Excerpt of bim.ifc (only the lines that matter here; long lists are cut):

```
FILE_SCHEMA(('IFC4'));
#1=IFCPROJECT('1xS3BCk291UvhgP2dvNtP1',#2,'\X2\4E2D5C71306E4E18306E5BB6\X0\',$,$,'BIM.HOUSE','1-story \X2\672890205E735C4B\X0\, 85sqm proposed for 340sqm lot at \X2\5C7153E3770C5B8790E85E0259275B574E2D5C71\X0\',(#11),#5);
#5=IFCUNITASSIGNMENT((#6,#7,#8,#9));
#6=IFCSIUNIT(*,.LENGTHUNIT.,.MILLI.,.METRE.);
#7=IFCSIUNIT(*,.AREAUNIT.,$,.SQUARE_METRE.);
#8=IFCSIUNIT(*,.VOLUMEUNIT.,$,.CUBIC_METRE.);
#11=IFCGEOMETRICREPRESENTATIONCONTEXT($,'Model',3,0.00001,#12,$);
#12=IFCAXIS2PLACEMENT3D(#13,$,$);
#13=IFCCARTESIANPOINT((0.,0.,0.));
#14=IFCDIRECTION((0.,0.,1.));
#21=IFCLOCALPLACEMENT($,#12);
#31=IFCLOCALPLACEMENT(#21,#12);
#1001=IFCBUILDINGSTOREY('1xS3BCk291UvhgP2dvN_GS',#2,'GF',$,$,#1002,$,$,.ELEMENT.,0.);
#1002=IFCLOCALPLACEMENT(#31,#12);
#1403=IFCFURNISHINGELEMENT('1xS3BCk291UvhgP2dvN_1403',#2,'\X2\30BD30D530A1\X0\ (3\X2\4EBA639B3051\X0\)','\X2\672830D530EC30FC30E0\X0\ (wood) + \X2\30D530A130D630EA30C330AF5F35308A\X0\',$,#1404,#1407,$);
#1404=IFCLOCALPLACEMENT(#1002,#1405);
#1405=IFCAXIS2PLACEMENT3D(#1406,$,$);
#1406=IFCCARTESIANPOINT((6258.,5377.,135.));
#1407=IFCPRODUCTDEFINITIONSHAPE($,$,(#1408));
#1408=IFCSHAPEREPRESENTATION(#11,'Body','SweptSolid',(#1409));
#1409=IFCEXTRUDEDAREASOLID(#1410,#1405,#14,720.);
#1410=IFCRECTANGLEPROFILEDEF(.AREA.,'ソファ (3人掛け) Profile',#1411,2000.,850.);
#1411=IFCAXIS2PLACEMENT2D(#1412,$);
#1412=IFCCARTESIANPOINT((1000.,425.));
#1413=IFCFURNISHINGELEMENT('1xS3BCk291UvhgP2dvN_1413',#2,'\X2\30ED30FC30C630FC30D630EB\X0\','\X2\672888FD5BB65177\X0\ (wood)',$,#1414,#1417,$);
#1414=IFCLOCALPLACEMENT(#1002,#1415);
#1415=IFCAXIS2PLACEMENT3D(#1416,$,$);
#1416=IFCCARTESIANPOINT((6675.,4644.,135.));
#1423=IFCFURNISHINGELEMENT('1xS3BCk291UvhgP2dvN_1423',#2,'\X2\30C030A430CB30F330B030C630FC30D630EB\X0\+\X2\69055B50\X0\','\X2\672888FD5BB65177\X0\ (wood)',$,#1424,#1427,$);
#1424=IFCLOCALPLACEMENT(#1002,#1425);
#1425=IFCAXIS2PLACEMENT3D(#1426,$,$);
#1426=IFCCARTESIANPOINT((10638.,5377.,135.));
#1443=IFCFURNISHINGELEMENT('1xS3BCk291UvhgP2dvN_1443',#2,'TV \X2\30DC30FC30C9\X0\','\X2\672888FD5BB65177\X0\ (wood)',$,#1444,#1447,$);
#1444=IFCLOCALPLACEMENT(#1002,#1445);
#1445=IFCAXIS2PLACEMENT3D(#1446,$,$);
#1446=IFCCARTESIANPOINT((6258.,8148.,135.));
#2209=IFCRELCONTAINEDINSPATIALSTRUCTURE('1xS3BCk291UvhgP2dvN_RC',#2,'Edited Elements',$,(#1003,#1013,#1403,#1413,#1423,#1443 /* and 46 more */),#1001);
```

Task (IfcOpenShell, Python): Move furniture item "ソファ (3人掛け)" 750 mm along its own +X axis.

```python
import ifcopenshell
import ifcopenshell.api.geometry
import ifcopenshell.util.placement

model = ifcopenshell.open("bim.ifc")

item = model.by_guid("1xS3BCk291UvhgP2dvN_1403")
matrix = ifcopenshell.util.placement.get_local_placement(item.ObjectPlacement)
matrix[:3, 3] += matrix[:3, 0] * 750.0
ifcopenshell.api.geometry.edit_object_placement(model, product=item, matrix=matrix, is_si=False)

print(ifcopenshell.util.placement.get_local_placement(item.ObjectPlacement).round(3) + 0.0)

model.write("bim_updated.ifc")
```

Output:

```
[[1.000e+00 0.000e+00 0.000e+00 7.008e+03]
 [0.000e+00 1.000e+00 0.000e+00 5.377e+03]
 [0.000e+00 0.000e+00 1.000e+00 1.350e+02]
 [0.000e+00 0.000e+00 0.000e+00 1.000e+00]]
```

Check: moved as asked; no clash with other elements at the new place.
